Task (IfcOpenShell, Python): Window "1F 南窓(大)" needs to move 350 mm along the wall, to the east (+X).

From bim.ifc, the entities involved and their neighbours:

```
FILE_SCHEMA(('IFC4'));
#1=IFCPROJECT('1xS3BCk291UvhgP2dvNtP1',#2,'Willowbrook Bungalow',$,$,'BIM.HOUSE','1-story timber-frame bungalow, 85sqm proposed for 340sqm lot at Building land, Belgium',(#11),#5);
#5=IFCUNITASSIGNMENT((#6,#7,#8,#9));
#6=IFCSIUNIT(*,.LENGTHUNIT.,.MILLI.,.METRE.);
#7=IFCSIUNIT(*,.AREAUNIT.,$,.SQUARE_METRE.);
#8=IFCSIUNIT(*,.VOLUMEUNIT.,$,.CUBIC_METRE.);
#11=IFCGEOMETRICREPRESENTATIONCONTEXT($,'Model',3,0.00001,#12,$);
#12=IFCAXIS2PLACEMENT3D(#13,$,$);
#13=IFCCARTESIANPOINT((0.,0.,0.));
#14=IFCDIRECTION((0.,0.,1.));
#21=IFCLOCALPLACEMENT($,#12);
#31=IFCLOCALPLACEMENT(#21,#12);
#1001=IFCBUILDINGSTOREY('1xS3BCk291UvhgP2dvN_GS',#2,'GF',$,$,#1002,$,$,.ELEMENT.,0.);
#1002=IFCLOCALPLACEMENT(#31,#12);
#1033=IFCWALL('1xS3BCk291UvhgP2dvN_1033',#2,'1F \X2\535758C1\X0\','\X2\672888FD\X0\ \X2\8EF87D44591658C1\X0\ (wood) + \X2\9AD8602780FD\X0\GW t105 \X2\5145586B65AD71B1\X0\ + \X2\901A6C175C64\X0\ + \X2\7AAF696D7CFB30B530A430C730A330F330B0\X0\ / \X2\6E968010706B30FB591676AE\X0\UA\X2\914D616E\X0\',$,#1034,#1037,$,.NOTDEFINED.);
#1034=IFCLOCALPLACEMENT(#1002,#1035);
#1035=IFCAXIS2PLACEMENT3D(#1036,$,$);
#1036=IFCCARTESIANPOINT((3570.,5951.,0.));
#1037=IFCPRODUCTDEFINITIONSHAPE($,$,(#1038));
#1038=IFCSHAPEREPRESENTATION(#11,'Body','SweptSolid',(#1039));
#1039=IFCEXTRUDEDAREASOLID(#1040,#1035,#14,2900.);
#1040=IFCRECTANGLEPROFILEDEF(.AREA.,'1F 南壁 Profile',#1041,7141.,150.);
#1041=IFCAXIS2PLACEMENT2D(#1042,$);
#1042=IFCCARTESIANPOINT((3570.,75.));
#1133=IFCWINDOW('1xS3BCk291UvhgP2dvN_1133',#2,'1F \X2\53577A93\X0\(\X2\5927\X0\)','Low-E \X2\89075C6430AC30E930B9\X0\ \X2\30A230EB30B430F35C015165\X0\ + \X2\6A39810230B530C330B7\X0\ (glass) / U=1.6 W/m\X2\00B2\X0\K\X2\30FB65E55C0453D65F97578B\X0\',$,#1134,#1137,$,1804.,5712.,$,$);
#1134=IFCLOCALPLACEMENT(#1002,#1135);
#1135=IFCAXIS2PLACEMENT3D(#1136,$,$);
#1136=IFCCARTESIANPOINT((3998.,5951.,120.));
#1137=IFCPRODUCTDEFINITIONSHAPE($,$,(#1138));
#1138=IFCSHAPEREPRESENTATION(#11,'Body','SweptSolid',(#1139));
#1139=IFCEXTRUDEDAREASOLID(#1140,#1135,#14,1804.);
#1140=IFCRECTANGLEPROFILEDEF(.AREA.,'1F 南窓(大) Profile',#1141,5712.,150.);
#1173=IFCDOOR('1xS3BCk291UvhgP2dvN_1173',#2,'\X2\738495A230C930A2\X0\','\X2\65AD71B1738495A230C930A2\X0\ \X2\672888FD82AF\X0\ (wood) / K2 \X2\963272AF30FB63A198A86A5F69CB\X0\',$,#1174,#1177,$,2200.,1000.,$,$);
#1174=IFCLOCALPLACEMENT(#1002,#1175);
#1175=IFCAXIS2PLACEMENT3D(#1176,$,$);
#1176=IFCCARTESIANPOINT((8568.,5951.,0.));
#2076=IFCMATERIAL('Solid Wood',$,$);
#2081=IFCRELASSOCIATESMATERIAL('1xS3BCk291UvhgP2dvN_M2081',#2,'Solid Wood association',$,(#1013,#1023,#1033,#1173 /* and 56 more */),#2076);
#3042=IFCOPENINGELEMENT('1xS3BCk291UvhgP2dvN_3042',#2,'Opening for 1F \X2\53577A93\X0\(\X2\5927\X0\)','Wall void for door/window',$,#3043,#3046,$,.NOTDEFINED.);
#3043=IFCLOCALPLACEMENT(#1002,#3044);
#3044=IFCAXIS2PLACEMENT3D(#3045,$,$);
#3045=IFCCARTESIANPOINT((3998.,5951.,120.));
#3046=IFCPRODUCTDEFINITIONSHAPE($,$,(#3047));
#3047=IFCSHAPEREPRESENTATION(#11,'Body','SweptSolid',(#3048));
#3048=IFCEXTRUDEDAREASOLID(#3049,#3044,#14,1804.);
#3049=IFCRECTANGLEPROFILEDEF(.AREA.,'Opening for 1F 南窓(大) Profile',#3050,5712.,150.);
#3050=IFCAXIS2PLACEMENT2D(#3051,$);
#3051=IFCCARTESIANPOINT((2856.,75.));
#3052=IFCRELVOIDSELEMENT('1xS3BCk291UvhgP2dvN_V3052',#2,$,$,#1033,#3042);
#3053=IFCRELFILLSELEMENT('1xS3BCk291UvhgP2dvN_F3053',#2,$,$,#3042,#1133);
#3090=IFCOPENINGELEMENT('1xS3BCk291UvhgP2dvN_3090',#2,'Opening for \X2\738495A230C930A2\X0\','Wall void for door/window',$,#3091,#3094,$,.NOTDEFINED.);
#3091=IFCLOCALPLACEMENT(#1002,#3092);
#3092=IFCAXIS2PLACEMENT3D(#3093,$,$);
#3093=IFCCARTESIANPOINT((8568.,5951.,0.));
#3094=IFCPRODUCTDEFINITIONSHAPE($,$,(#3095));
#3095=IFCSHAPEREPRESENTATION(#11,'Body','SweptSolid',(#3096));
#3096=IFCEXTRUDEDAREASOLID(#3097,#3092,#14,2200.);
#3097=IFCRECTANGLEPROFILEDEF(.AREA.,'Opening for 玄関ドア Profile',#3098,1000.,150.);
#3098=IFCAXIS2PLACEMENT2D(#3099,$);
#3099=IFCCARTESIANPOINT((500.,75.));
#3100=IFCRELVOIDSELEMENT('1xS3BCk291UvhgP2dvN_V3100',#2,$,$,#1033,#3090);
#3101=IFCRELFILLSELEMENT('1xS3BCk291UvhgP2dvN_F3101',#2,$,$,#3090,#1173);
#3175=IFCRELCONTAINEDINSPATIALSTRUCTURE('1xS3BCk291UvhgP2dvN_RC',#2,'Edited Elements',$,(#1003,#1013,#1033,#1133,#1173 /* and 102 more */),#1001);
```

```python
import ifcopenshell
import ifcopenshell.api.geometry
import ifcopenshell.util.placement
import ifcopenshell.util.unit

model = ifcopenshell.open("bim.ifc")
unit_scale = ifcopenshell.util.unit.calculate_unit_scale(model)

window = model.by_guid("1xS3BCk291UvhgP2dvN_1133")
opening = window.FillsVoids[0].RelatingOpeningElement
wall = opening.VoidsElements[0].RelatingBuildingElement

wall_matrix = ifcopenshell.util.placement.get_local_placement(wall.ObjectPlacement)
shift = wall_matrix[:3, 0] * 0.35 / unit_scale
before = ifcopenshell.util.placement.get_local_placement(window.ObjectPlacement)[:3, 3].copy()

# The window is not placed relative to its opening, so move both.
for product in (opening, window):
    matrix = ifcopenshell.util.placement.get_local_placement(product.ObjectPlacement)
    matrix[:3, 3] += shift
    ifcopenshell.api.geometry.edit_object_placement(model, product=product, matrix=matrix, is_si=False)

after = ifcopenshell.util.placement.get_local_placement(window.ObjectPlacement)[:3, 3]
print("window moved by", (after - before).round(3) + 0.0)

model.write("bim_v2.ifc")
```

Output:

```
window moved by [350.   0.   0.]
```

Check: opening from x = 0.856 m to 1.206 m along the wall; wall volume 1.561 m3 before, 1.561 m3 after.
